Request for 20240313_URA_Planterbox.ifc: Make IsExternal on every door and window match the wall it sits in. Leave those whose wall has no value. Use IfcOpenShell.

First a look at what the model holds.

```python
import ifcopenshell
import ifcopenshell.util.element

model = ifcopenshell.open("20240313_URA_Planterbox.ifc")
print(model.schema)
seen = {}
for e in model.by_type("IfcDoor") + model.by_type("IfcWindow"):
    if not e.FillsVoids:
        continue
    host = e.FillsVoids[0].RelatingOpeningElement.VoidsElements[0].RelatingBuildingElement
    own = ifcopenshell.util.element.get_pset(e, f"Pset_{e.is_a()[3:].removesuffix('StandardCase')}Common", "IsExternal")
    wall = ifcopenshell.util.element.get_pset(host, "Pset_WallCommon", "IsExternal")
    seen[e.is_a(), own, wall] = seen.get((e.is_a(), own, wall), 0) + 1
for (cls, own, wall), count in sorted(seen.items(), key=str):
    print(count, cls, "IsExternal:", own, "| host wall:", wall)
```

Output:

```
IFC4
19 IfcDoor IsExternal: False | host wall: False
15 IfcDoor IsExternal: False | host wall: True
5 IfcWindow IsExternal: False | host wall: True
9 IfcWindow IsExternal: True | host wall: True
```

```python
import ifcopenshell
import ifcopenshell.api.pset
import ifcopenshell.util.element

model = ifcopenshell.open("20240313_URA_Planterbox.ifc")

count = 0
for ifc_class, pset_name in (("IfcDoor", "Pset_DoorCommon"), ("IfcWindow", "Pset_WindowCommon")):
    for e in model.by_type(ifc_class):
        if not e.FillsVoids:
            continue
        host = e.FillsVoids[0].RelatingOpeningElement.VoidsElements[0].RelatingBuildingElement
        external = ifcopenshell.util.element.get_pset(host, "Pset_WallCommon", "IsExternal")
        if external is None or ifcopenshell.util.element.get_pset(e, pset_name, "IsExternal") == external:
            continue
        pset = ifcopenshell.api.pset.add_pset(model, product=e, name=pset_name)
        ifcopenshell.api.pset.edit_pset(model, pset=pset, properties={"IsExternal": external})
        count += 1

print(count, "updated")

model.write("20240313_URA_Planterbox_edited.ifc")
```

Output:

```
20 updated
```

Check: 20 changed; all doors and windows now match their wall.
